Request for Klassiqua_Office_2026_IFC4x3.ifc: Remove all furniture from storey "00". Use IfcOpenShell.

First a look at what the model holds.

```python
import ifcopenshell
import ifcopenshell.util.element

model = ifcopenshell.open("Klassiqua_Office_2026_IFC4x3.ifc")
print(model.schema)
storey = next(s for s in model.by_type("IfcBuildingStorey") if s.Name == "00")
furniture = [e for e in ifcopenshell.util.element.get_decomposition(storey) if e.is_a("IfcFurnishingElement")]
seen = {}
for e in furniture:
    element_type = ifcopenshell.util.element.get_type(e)
    name = element_type.Name if element_type not in (None, e) else None
    seen[name] = seen.get(name, 0) + 1
for name, count in sorted(seen.items(), key=str):
    print(count, "x", name)
```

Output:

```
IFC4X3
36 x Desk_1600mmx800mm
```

```python
import ifcopenshell
import ifcopenshell.api.root
import ifcopenshell.util.element

model = ifcopenshell.open("Klassiqua_Office_2026_IFC4x3.ifc")

storey = next(s for s in model.by_type("IfcBuildingStorey") if s.Name == "00")
furniture = [e for e in ifcopenshell.util.element.get_decomposition(storey) if e.is_a("IfcFurnishingElement")]

for e in furniture:
    ifcopenshell.api.root.remove_product(model, product=e)
print(len(furniture), "removed")

model.write("Klassiqua_Office_2026_IFC4x3_rev.ifc")
```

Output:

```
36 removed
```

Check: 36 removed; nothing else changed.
